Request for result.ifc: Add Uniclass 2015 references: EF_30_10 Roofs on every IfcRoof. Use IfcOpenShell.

First a look at what the model holds.

```python
import ifcopenshell

model = ifcopenshell.open("result.ifc")
print(model.schema)
print("classifications:", [c.Name for c in model.by_type("IfcClassification")])
for ifc_class in ("IfcDoor", "IfcRoof", "IfcStair", "IfcWall", "IfcWindow"):
    print(ifc_class, len(model.by_type(ifc_class)))
```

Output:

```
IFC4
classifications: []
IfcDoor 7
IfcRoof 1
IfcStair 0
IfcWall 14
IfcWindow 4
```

```python
import ifcopenshell
import ifcopenshell.api.classification

model = ifcopenshell.open("result.ifc")

system = ifcopenshell.api.classification.add_classification(model, classification="Uniclass 2015")

codes = {
    "IfcRoof": ("EF_30_10", "Roofs"),
}
for ifc_class, (code, name) in codes.items():
    products = model.by_type(ifc_class)
    ifcopenshell.api.classification.add_reference(
        model, products=products, classification=system, identification=code, name=name
    )
    print(code, len(products))

model.write("result_updated.ifc")
```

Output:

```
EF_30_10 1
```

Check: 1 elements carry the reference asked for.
